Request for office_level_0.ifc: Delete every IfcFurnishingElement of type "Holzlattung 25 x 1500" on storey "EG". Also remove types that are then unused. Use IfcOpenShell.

First a look at what the model holds.

```python
import ifcopenshell
import ifcopenshell.util.element

model = ifcopenshell.open("office_level_0.ifc")
print(model.schema)
storey = next(s for s in model.by_type("IfcBuildingStorey") if s.Name == "EG")
furniture = [e for e in ifcopenshell.util.element.get_decomposition(storey) if e.is_a("IfcFurnishingElement")]
seen = {}
for e in furniture:
    element_type = ifcopenshell.util.element.get_type(e)
    name = element_type.Name if element_type not in (None, e) else None
    seen[name] = seen.get(name, 0) + 1
for name, count in sorted(seen.items(), key=str):
    print(count, "x", name)
```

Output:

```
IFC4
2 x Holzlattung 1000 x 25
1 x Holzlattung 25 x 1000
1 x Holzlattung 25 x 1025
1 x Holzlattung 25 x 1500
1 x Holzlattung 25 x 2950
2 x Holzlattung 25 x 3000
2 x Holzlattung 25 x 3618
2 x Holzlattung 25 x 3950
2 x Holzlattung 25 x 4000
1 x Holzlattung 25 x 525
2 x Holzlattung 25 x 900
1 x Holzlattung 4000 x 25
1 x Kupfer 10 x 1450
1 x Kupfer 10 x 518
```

```python
import ifcopenshell
import ifcopenshell.api.root
import ifcopenshell.util.element

model = ifcopenshell.open("office_level_0.ifc")

storey = next(s for s in model.by_type("IfcBuildingStorey") if s.Name == "EG")
furniture = [e for e in ifcopenshell.util.element.get_decomposition(storey) if e.is_a("IfcFurnishingElement")]
targets = [e for e in furniture if (t := ifcopenshell.util.element.get_type(e)) not in (None, e) and t.Name == "Holzlattung 25 x 1500"]
types = {ifcopenshell.util.element.get_type(e) for e in targets} - {None, *targets}

for e in targets:
    ifcopenshell.api.root.remove_product(model, product=e)
print(len(targets), "removed")

unused = [t for t in types if not ifcopenshell.util.element.get_types(t)]
for t in unused:
    ifcopenshell.api.root.remove_product(model, product=t)
print(len(unused), "unused types removed")

model.write("office_level_0-out.ifc")
```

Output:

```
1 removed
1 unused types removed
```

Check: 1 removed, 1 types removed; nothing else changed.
